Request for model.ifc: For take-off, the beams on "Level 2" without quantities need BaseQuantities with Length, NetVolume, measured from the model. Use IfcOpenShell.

First a look at what the model holds.

```python
import ifcopenshell
import ifcopenshell.util.element
import ifcopenshell.util.unit

model = ifcopenshell.open("model.ifc")
print(model.schema)
for unit_type in ("LENGTHUNIT", "AREAUNIT", "VOLUMEUNIT"):
    print(unit_type, ifcopenshell.util.unit.calculate_unit_scale(model, unit_type))
storey = next(s for s in model.by_type("IfcBuildingStorey") if s.Name == "Level 2")
beams = [e for e in ifcopenshell.util.element.get_decomposition(storey) if e.is_a("IfcBeam")]
for e in sorted(beams, key=lambda e: e.id()):
    print(e.id(), e.is_a(), e.Name, list(ifcopenshell.util.element.get_psets(e, qtos_only=True)), sep=" | ")
```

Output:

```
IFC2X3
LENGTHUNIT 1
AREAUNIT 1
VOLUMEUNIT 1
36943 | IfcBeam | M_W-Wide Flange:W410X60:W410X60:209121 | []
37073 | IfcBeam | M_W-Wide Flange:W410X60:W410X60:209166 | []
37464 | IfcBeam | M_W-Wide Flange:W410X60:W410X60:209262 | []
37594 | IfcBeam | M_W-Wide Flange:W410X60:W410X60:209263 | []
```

```python
import ifcopenshell
import ifcopenshell.api.pset
import ifcopenshell.geom
import ifcopenshell.util.element
import ifcopenshell.util.shape
import ifcopenshell.util.unit

model = ifcopenshell.open("model.ifc")
unit_scale = ifcopenshell.util.unit.calculate_unit_scale(model)
volume_scale = ifcopenshell.util.unit.calculate_unit_scale(model, "VOLUMEUNIT")
settings = ifcopenshell.geom.settings()

storey = next(s for s in model.by_type("IfcBuildingStorey") if s.Name == "Level 2")
beams = [e for e in ifcopenshell.util.element.get_decomposition(storey) if e.is_a("IfcBeam")]

for e in sorted(beams, key=lambda e: e.id()):
    if ifcopenshell.util.element.get_psets(e, qtos_only=True, should_inherit=False):
        continue
    # Geometry comes back in metres, in the element's own axes.
    shape = ifcopenshell.geom.create_shape(settings, e)
    values = {
        "Length": ifcopenshell.util.shape.get_max_xyz(shape.geometry) / unit_scale,
        "NetVolume": ifcopenshell.util.shape.get_volume(shape.geometry) / volume_scale,
    }
    qto = ifcopenshell.api.pset.add_qto(model, product=e, name="BaseQuantities")
    ifcopenshell.api.pset.edit_qto(model, qto=qto, properties=values)
    print(e.id(), {k: round(v, 3) for k, v in values.items()})

model.write("model_v2.ifc")
```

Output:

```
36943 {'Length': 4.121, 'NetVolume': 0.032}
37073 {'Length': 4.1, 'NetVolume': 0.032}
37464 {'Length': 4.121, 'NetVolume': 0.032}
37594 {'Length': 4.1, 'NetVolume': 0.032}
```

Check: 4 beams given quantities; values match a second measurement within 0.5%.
